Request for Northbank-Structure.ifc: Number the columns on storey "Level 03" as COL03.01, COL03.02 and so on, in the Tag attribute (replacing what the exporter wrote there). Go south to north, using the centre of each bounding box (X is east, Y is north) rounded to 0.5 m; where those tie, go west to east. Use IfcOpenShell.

First a look at what the model holds.

```python
import ifcopenshell
import ifcopenshell.util.element
import ifcopenshell.util.placement

model = ifcopenshell.open("Northbank-Structure.ifc")
print(model.schema)
storey = next(s for s in model.by_type("IfcBuildingStorey") if s.Name == "Level 03")
columns = [e for e in ifcopenshell.util.element.get_decomposition(storey) if e.is_a("IfcColumn")]
for e in sorted(columns, key=lambda e: e.id()):
    origin = ifcopenshell.util.placement.get_local_placement(e.ObjectPlacement)[:3, 3]
    print(e.id(), e.Tag, e.Name, origin.round(2) + 0.0, sep=" | ")
```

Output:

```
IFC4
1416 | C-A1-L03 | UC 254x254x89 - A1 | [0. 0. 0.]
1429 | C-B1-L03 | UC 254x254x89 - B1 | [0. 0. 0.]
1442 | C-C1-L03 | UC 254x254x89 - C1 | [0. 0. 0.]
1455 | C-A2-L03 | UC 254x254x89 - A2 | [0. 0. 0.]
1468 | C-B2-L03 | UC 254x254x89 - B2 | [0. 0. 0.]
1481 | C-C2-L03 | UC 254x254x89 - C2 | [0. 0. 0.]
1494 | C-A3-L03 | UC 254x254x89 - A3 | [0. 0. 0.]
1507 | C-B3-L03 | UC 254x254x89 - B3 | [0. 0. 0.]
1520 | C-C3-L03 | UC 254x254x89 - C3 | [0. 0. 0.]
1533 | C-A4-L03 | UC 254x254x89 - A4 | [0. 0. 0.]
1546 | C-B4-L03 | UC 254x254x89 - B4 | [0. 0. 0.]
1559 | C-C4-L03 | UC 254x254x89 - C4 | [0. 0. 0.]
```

```python
import ifcopenshell
import ifcopenshell.geom
import ifcopenshell.util.element
import ifcopenshell.util.shape

model = ifcopenshell.open("Northbank-Structure.ifc")
settings = ifcopenshell.geom.settings()
settings.set("use-world-coords", True)


def centre(element):
    shape = ifcopenshell.geom.create_shape(settings, element)
    return ifcopenshell.util.shape.get_bbox_centroid(shape.geometry)


storey = next(s for s in model.by_type("IfcBuildingStorey") if s.Name == "Level 03")
columns = [e for e in ifcopenshell.util.element.get_decomposition(storey) if e.is_a("IfcColumn")]

# Insertion points can sit at a corner or the storey origin, so sort by the geometry (in metres).
centres = {e: centre(e) for e in columns}
columns.sort(key=lambda e: (round(centres[e][1] / 0.5), centres[e][0]))

for i, e in enumerate(columns, start=1):
    number = f"COL03.{i:02d}"
    e.Tag = number
    print(e.id(), number)

model.write("Northbank-Structure_v2.ifc")
```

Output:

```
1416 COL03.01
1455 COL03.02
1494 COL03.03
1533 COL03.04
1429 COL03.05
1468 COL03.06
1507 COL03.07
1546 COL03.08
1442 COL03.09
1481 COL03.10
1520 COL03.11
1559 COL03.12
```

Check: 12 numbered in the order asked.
